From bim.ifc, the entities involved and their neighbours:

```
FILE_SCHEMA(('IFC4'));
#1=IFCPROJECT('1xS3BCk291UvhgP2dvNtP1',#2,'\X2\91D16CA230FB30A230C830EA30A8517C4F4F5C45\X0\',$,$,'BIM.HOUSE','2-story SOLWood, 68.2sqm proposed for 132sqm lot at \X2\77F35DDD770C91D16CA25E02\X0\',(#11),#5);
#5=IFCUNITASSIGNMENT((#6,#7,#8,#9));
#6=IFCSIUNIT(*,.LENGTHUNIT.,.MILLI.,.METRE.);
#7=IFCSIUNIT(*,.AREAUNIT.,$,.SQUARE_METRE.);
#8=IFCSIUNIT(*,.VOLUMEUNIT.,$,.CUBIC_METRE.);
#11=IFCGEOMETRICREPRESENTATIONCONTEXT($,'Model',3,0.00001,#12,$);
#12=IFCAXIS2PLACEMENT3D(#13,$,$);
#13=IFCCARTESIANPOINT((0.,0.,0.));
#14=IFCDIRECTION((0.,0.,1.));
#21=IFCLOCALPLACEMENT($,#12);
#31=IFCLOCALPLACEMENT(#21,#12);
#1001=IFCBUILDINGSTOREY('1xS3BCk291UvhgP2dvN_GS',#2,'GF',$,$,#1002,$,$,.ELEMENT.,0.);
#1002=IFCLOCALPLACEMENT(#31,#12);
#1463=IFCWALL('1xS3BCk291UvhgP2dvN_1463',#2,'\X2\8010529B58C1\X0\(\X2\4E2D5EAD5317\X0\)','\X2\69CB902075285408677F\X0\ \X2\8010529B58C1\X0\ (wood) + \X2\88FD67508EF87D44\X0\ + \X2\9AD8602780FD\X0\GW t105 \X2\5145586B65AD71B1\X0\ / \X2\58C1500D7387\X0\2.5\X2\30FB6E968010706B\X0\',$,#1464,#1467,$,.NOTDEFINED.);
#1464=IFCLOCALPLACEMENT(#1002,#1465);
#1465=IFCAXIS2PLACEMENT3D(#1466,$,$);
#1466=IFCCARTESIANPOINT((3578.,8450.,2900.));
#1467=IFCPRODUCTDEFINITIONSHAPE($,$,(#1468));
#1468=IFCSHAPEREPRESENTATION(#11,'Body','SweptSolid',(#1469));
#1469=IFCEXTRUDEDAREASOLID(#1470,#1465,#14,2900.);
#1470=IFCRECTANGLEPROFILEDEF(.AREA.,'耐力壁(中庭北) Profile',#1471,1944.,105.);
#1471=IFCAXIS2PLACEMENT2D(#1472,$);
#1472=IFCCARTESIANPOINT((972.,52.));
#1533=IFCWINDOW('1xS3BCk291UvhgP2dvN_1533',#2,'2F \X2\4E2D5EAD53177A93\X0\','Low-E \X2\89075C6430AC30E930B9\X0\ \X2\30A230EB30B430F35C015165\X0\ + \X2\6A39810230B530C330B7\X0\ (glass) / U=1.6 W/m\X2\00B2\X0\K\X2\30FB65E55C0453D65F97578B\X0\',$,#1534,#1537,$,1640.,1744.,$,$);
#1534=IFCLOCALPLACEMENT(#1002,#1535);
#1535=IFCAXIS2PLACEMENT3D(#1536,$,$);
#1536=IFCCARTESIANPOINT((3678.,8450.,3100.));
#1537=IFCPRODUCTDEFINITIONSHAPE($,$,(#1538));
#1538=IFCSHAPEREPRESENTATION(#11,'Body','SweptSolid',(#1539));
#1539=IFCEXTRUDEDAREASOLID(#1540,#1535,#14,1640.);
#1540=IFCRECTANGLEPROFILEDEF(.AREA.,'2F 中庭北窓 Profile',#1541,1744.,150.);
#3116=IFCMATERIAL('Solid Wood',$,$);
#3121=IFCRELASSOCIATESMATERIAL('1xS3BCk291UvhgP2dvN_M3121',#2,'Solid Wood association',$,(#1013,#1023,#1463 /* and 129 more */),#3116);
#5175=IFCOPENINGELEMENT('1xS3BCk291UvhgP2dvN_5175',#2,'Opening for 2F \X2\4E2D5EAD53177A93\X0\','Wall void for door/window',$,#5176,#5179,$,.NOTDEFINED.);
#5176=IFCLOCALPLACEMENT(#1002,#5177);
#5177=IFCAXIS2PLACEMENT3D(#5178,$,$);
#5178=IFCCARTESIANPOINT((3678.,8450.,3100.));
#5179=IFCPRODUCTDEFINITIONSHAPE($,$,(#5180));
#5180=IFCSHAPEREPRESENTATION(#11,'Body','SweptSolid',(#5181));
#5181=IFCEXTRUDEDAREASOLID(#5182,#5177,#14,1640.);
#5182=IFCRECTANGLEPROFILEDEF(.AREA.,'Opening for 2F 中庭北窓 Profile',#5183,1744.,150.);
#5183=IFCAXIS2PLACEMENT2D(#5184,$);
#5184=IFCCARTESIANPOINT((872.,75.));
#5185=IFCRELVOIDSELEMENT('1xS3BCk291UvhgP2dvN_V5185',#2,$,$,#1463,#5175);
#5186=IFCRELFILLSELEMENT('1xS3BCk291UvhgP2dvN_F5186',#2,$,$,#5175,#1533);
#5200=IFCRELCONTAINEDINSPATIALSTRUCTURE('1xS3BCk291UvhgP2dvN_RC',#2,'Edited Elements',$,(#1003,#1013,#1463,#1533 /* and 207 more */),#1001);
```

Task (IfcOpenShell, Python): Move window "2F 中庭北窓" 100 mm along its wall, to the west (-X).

```python
import ifcopenshell
import ifcopenshell.api.geometry
import ifcopenshell.util.placement
import ifcopenshell.util.unit

model = ifcopenshell.open("bim.ifc")
unit_scale = ifcopenshell.util.unit.calculate_unit_scale(model)

window = model.by_guid("1xS3BCk291UvhgP2dvN_1533")
opening = window.FillsVoids[0].RelatingOpeningElement
wall = opening.VoidsElements[0].RelatingBuildingElement

wall_matrix = ifcopenshell.util.placement.get_local_placement(wall.ObjectPlacement)
shift = wall_matrix[:3, 0] * -0.1 / unit_scale
before = ifcopenshell.util.placement.get_local_placement(window.ObjectPlacement)[:3, 3].copy()

# The window is not placed relative to its opening, so move both.
for product in (opening, window):
    matrix = ifcopenshell.util.placement.get_local_placement(product.ObjectPlacement)
    matrix[:3, 3] += shift
    ifcopenshell.api.geometry.edit_object_placement(model, product=product, matrix=matrix, is_si=False)

after = ifcopenshell.util.placement.get_local_placement(window.ObjectPlacement)[:3, 3]
print("window moved by", (after - before).round(3) + 0.0)

model.write("bim-out.ifc")
```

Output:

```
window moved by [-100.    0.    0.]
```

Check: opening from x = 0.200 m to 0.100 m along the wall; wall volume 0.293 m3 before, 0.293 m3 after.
